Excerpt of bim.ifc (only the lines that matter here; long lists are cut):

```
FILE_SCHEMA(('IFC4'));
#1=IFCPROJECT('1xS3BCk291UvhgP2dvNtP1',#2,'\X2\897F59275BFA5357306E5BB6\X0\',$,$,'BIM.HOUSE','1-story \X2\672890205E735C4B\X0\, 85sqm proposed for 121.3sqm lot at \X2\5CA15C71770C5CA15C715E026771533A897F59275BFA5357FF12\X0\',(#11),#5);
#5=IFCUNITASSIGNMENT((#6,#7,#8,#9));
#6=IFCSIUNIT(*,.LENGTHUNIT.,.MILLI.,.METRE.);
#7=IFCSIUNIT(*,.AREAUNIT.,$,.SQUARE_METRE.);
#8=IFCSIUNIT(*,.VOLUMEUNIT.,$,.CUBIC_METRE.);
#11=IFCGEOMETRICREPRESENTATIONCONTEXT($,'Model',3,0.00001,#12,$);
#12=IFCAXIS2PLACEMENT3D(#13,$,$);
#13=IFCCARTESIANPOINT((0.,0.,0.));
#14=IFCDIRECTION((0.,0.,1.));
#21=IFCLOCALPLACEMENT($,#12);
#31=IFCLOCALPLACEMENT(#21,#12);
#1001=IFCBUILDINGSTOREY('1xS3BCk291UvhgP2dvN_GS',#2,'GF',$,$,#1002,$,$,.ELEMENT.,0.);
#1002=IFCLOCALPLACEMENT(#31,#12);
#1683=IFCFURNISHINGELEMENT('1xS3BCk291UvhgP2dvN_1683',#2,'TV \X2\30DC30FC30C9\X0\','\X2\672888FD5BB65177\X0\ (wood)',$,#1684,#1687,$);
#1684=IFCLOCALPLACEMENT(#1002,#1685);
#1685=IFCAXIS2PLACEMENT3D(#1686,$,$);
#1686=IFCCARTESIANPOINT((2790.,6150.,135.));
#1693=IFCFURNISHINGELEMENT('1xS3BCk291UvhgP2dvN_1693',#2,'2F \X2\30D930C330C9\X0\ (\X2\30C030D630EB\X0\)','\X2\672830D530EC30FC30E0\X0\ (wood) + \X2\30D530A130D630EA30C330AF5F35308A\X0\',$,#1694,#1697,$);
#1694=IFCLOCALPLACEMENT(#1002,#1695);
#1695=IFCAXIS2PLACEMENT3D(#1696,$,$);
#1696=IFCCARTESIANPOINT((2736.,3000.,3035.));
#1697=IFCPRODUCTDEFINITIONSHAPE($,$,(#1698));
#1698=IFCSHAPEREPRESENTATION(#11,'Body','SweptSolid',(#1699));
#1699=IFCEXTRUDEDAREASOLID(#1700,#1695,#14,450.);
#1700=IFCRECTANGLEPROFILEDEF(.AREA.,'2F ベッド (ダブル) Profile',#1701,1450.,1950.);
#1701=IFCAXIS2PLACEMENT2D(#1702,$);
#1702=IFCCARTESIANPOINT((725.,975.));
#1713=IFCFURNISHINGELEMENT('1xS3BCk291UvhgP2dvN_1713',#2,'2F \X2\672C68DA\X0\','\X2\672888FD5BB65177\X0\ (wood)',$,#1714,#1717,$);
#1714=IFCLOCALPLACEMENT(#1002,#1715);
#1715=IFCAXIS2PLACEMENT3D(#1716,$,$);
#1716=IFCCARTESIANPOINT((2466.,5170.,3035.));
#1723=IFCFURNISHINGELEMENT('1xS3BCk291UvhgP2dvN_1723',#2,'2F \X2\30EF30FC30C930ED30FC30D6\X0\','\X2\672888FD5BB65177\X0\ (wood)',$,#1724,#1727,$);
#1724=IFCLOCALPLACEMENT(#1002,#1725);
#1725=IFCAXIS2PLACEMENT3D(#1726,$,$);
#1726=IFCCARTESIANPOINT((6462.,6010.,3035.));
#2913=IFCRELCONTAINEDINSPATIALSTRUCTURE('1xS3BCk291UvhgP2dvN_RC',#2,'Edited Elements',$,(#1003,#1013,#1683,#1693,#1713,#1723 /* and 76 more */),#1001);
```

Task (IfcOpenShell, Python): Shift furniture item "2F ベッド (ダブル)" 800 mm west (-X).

```python
import ifcopenshell
import ifcopenshell.api.geometry
import ifcopenshell.util.placement
import ifcopenshell.util.unit

model = ifcopenshell.open("bim.ifc")
unit_scale = ifcopenshell.util.unit.calculate_unit_scale(model)

item = model.by_guid("1xS3BCk291UvhgP2dvN_1693")
matrix = ifcopenshell.util.placement.get_local_placement(item.ObjectPlacement)
matrix[0, 3] -= 0.8 / unit_scale
ifcopenshell.api.geometry.edit_object_placement(model, product=item, matrix=matrix, is_si=False)

print(ifcopenshell.util.placement.get_local_placement(item.ObjectPlacement).round(3) + 0.0)

model.write("bim_edited.ifc")
```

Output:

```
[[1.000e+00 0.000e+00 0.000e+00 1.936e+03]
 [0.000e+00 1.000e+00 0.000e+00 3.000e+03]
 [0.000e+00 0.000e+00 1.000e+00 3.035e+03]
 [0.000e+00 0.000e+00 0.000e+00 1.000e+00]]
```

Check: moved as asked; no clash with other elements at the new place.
